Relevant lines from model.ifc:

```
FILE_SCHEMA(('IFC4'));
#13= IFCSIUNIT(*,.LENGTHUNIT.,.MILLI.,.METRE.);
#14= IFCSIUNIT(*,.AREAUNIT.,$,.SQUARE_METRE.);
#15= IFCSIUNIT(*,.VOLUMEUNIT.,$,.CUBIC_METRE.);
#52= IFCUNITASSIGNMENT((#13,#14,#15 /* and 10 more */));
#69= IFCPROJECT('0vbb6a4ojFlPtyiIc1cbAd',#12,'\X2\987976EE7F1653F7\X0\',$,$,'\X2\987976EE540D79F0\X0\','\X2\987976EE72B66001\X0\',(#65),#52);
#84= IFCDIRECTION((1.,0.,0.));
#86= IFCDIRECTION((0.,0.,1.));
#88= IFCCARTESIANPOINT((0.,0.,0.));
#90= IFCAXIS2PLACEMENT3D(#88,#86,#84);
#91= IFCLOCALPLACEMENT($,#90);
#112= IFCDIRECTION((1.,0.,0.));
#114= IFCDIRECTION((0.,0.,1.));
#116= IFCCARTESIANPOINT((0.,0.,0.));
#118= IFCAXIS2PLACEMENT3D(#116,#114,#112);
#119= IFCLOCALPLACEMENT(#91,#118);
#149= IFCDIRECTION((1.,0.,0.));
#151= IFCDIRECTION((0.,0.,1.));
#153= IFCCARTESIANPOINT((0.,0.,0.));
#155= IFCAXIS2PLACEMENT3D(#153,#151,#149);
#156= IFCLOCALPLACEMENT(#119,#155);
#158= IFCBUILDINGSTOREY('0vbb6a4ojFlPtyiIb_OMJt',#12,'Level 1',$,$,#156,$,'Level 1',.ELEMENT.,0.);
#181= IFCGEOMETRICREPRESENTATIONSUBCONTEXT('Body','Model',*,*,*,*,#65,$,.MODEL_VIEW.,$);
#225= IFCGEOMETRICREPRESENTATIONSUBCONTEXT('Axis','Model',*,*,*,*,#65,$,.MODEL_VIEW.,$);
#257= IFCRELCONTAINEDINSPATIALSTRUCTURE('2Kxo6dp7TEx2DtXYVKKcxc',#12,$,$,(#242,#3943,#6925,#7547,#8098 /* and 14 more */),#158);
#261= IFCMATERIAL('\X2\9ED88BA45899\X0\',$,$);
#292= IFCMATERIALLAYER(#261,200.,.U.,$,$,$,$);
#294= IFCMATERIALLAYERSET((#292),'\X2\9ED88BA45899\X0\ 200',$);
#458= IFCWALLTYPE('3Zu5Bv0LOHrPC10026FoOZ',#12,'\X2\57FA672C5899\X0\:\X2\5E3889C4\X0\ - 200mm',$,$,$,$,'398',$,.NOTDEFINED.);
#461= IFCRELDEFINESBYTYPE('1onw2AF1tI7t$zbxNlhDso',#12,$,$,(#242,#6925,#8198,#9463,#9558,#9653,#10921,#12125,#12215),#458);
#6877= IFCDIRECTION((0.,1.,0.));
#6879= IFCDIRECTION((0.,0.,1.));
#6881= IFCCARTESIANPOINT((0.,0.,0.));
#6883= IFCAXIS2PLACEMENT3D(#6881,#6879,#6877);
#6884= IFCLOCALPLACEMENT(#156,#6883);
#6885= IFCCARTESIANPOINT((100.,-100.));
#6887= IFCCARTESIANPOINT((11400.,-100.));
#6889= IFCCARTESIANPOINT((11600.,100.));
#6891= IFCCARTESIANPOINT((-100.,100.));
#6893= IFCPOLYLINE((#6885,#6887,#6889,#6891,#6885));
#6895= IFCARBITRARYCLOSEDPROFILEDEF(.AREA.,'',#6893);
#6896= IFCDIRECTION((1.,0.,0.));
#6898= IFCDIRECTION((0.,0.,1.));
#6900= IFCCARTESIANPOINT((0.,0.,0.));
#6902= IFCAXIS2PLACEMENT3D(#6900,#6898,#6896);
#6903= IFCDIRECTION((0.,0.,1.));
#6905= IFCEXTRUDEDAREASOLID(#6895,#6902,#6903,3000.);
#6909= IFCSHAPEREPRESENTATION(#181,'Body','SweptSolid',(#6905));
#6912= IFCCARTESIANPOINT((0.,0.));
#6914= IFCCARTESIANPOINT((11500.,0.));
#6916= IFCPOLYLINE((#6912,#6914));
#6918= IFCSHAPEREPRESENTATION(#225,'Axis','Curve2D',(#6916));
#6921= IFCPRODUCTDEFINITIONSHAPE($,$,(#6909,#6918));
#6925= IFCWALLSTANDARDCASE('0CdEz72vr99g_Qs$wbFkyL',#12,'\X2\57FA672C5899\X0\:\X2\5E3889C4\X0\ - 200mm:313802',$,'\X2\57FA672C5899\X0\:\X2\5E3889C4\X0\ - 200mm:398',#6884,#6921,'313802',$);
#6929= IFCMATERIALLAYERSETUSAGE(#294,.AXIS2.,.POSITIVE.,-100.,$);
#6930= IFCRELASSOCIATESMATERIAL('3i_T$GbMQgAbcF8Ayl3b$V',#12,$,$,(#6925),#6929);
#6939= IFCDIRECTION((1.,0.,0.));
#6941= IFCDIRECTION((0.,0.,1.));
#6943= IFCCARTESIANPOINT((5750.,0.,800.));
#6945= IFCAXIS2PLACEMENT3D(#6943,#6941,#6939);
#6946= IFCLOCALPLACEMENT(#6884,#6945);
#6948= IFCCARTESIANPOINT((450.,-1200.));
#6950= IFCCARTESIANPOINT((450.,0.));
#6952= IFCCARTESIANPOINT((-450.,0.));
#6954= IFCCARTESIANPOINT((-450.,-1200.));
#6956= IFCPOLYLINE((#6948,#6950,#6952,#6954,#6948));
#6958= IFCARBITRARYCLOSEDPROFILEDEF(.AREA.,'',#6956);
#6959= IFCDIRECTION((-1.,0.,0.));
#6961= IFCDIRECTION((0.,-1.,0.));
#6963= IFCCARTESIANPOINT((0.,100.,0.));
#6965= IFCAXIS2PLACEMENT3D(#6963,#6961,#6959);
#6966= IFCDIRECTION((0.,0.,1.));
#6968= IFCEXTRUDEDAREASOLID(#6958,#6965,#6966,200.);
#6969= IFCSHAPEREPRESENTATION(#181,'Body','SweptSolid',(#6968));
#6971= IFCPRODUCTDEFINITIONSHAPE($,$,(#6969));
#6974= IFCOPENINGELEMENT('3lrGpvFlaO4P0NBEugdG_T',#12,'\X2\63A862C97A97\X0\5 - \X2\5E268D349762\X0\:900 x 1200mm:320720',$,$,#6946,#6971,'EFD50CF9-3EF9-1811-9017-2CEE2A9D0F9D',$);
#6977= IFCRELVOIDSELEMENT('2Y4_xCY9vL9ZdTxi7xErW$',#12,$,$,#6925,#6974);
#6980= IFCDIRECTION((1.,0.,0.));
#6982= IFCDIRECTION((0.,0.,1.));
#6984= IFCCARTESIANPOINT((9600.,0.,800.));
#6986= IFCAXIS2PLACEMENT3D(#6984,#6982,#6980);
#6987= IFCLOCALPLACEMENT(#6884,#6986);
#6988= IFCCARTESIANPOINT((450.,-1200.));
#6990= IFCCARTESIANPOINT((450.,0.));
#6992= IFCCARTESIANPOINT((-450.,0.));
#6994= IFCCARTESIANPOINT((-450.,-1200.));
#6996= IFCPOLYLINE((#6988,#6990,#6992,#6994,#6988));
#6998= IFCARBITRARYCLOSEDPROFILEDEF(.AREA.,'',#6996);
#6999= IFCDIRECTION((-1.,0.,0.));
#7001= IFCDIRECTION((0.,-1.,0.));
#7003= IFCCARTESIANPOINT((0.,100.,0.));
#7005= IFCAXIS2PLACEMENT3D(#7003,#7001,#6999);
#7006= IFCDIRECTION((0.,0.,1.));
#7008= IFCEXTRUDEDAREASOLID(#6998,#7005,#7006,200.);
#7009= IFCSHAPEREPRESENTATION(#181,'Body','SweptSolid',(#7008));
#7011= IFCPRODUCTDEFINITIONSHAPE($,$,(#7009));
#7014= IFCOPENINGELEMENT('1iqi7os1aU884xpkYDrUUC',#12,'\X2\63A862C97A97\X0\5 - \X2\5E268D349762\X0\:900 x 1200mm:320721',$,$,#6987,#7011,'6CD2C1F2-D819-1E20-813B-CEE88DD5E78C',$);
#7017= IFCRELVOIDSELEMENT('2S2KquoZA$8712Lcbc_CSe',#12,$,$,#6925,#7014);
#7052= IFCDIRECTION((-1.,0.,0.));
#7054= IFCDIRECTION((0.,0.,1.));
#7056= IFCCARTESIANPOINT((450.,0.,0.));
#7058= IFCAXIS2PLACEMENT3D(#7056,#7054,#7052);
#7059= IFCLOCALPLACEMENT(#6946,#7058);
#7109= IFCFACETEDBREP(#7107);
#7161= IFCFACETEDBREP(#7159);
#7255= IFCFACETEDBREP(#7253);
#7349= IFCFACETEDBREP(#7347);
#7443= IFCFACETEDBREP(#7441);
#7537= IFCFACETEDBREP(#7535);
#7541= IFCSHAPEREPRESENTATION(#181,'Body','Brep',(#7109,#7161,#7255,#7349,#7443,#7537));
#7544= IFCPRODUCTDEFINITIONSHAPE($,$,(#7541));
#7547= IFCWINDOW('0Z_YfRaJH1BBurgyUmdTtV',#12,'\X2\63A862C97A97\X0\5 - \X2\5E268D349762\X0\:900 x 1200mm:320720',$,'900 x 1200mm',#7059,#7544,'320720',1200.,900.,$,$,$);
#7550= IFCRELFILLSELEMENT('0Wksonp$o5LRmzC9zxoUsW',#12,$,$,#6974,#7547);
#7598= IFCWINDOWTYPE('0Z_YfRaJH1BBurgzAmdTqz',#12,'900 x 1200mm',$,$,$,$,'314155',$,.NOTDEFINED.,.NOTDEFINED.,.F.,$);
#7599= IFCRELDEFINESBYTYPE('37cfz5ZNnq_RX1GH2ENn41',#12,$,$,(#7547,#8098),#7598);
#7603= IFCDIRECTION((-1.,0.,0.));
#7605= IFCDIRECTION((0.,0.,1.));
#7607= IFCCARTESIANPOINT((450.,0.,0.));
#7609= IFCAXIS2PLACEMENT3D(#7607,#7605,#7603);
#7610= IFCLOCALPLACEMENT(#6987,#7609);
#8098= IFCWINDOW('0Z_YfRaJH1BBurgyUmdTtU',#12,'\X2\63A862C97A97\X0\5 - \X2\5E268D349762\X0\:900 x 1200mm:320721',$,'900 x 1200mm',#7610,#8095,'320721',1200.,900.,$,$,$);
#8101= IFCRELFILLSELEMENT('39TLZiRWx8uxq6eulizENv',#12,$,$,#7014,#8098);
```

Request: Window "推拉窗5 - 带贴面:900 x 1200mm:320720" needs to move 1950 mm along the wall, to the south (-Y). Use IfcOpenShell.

```python
import ifcopenshell
import ifcopenshell.api.geometry
import ifcopenshell.util.placement

model = ifcopenshell.open("model.ifc")

window = model.by_guid("0Z_YfRaJH1BBurgyUmdTtV")
opening = window.FillsVoids[0].RelatingOpeningElement
wall = opening.VoidsElements[0].RelatingBuildingElement

wall_matrix = ifcopenshell.util.placement.get_local_placement(wall.ObjectPlacement)
shift = wall_matrix[:3, 0] * -1950.0
before = ifcopenshell.util.placement.get_local_placement(window.ObjectPlacement)[:3, 3].copy()

# The window is placed relative to its opening, so it follows when the opening moves.
matrix = ifcopenshell.util.placement.get_local_placement(opening.ObjectPlacement)
matrix[:3, 3] += shift
ifcopenshell.api.geometry.edit_object_placement(
    model, product=opening, matrix=matrix, is_si=False, should_transform_children=True
)

after = ifcopenshell.util.placement.get_local_placement(window.ObjectPlacement)[:3, 3]
print("window moved by", (after - before).round(3) + 0.0)

model.write("model_v2.ifc")
```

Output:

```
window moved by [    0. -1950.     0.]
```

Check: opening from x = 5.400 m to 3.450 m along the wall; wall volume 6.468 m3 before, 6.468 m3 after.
